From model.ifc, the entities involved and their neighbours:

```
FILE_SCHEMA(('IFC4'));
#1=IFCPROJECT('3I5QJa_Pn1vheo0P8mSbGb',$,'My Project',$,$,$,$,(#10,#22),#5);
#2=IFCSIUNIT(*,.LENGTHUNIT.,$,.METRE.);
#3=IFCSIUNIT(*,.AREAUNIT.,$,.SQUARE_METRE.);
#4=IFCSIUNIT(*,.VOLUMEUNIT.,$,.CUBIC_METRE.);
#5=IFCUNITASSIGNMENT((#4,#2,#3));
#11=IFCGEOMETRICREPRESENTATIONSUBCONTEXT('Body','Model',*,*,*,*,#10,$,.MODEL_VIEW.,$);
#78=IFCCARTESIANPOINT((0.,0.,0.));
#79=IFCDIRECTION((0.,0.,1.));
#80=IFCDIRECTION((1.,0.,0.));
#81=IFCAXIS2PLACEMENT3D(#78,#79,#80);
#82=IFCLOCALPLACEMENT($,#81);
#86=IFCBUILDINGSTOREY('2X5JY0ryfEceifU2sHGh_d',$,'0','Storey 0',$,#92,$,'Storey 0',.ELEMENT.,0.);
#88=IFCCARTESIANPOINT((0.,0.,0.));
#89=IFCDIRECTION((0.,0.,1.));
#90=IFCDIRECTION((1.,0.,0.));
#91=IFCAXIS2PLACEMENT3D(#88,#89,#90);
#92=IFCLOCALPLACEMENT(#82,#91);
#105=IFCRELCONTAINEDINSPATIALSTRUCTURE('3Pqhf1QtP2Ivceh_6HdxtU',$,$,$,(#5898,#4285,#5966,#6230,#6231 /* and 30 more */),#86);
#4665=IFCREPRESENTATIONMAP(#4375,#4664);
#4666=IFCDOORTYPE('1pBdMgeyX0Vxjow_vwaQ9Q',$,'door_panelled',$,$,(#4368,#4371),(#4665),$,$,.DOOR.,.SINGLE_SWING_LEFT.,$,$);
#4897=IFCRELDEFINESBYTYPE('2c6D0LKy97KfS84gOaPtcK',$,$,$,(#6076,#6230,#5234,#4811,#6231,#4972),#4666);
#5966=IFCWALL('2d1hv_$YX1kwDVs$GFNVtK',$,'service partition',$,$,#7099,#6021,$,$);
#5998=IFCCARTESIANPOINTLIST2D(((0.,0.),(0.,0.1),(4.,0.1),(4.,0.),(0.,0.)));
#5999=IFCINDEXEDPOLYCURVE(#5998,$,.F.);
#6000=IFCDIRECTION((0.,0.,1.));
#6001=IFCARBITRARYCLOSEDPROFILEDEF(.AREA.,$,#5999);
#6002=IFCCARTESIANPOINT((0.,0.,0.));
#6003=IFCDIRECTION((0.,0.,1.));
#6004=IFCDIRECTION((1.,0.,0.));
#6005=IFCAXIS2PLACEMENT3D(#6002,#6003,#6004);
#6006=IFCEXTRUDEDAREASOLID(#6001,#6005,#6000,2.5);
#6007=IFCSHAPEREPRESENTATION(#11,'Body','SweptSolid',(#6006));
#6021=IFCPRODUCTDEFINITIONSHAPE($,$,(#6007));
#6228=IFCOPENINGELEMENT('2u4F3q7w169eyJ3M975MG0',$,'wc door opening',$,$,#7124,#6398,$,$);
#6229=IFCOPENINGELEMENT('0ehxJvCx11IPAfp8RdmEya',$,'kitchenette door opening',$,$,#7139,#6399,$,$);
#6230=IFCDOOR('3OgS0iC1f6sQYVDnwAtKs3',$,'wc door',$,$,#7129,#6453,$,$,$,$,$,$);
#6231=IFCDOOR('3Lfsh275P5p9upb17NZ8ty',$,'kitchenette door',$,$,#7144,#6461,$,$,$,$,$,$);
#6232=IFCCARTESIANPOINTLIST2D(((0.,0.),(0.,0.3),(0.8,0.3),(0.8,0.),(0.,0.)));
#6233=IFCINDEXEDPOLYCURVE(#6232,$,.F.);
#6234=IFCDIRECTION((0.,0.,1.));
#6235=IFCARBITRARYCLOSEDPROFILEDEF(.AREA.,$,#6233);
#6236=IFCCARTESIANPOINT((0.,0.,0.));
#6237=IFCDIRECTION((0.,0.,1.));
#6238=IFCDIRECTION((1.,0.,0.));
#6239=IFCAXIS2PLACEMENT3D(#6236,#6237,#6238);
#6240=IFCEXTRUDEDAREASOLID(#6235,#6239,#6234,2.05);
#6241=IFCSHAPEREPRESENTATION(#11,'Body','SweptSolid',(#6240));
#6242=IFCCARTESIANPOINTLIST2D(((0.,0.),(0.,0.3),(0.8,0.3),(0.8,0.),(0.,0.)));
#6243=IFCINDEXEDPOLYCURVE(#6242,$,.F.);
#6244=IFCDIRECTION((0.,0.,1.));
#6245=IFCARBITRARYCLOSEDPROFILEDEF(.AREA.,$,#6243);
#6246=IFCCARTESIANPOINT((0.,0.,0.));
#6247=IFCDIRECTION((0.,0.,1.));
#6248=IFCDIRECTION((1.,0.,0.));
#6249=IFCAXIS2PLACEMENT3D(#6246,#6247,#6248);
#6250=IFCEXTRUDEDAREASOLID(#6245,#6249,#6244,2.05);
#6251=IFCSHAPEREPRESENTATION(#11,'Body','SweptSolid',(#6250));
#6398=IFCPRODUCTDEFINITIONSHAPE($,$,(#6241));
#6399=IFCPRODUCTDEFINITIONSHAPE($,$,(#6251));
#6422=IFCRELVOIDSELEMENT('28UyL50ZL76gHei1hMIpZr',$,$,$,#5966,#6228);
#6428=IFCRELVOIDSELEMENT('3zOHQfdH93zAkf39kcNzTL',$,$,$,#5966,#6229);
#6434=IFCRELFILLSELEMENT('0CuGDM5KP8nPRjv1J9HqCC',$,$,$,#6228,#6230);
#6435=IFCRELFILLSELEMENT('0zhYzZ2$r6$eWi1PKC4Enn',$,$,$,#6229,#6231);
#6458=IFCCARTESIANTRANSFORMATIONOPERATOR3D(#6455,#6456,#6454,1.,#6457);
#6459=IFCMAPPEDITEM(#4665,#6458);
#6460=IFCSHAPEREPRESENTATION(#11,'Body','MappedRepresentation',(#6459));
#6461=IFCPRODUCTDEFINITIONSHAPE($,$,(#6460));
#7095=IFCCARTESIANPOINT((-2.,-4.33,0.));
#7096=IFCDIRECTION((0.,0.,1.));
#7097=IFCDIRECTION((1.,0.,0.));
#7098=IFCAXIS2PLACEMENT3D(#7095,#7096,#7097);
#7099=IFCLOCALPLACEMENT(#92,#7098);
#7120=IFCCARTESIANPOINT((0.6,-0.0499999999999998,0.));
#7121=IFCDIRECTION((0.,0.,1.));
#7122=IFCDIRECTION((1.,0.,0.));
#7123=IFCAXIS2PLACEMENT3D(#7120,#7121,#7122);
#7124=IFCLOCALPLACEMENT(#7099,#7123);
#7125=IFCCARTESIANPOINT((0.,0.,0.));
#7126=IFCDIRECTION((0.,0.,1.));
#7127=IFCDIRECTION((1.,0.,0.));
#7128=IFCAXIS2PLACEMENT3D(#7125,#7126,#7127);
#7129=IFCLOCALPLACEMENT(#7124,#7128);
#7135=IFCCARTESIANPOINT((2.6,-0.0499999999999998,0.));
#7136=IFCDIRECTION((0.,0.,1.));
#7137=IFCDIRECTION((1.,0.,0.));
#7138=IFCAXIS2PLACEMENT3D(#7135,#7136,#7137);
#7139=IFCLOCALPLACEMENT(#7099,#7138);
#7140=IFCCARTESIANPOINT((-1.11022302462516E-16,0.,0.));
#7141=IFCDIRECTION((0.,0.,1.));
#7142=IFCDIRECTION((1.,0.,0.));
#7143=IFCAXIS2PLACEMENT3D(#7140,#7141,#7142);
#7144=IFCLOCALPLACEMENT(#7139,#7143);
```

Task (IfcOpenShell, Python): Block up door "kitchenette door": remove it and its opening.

```python
import ifcopenshell
import ifcopenshell.api.feature
import ifcopenshell.api.root
import ifcopenshell.geom
import ifcopenshell.util.shape

model = ifcopenshell.open("model.ifc")
settings = ifcopenshell.geom.settings()


def volume(element):
    """Net volume in cubic metres, openings subtracted."""
    shape = ifcopenshell.geom.create_shape(settings, element)
    return ifcopenshell.util.shape.get_volume(shape.geometry)


door = model.by_guid("3Lfsh275P5p9upb17NZ8ty")
opening = door.FillsVoids[0].RelatingOpeningElement
wall = opening.VoidsElements[0].RelatingBuildingElement
before = volume(wall)

ifcopenshell.api.root.remove_product(model, product=door)
ifcopenshell.api.feature.remove_feature(model, feature=opening)

after = volume(wall)

print(f"wall volume {before:.3f} -> {after:.3f} m3")

model.write("model-out.ifc")
```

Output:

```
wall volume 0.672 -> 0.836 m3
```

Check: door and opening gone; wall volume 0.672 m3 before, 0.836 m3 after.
